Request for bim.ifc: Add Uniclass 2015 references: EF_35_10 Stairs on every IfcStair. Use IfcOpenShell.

First a look at what the model holds.

```python
import ifcopenshell

model = ifcopenshell.open("bim.ifc")
print(model.schema)
print("classifications:", [c.Name for c in model.by_type("IfcClassification")])
for ifc_class in ("IfcDoor", "IfcRoof", "IfcStair", "IfcWall", "IfcWindow"):
    print(ifc_class, len(model.by_type(ifc_class)))
```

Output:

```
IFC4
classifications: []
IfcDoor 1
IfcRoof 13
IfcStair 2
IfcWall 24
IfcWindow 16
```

```python
import ifcopenshell
import ifcopenshell.api.classification

model = ifcopenshell.open("bim.ifc")

system = ifcopenshell.api.classification.add_classification(model, classification="Uniclass 2015")

codes = {
    "IfcStair": ("EF_35_10", "Stairs"),
}
for ifc_class, (code, name) in codes.items():
    products = model.by_type(ifc_class)
    ifcopenshell.api.classification.add_reference(
        model, products=products, classification=system, identification=code, name=name
    )
    print(code, len(products))

model.write("bim_v2.ifc")
```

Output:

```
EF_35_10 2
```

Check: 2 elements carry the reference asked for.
